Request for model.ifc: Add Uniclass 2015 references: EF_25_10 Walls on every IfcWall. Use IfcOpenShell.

First a look at what the model holds.

```python
import ifcopenshell

model = ifcopenshell.open("model.ifc")
print(model.schema)
print("classifications:", [c.Name for c in model.by_type("IfcClassification")])
for ifc_class in ("IfcDoor", "IfcRoof", "IfcStair", "IfcWall", "IfcWindow"):
    print(ifc_class, len(model.by_type(ifc_class)))
```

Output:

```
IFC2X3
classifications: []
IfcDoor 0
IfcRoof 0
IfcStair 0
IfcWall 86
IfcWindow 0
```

```python
import ifcopenshell
import ifcopenshell.api.classification

model = ifcopenshell.open("model.ifc")

# IFC2X3 requires Source and Edition and has no link from the project to the system.
system = model.create_entity("IfcClassification", Source="NBS", Edition="2015", Name="Uniclass 2015")

codes = {
    "IfcWall": ("EF_25_10", "Walls"),
}
for ifc_class, (code, name) in codes.items():
    products = model.by_type(ifc_class)
    ifcopenshell.api.classification.add_reference(
        model, products=products, classification=system, identification=code, name=name
    )
    print(code, len(products))

model.write("model_updated.ifc")
```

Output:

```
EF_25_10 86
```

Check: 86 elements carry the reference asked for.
